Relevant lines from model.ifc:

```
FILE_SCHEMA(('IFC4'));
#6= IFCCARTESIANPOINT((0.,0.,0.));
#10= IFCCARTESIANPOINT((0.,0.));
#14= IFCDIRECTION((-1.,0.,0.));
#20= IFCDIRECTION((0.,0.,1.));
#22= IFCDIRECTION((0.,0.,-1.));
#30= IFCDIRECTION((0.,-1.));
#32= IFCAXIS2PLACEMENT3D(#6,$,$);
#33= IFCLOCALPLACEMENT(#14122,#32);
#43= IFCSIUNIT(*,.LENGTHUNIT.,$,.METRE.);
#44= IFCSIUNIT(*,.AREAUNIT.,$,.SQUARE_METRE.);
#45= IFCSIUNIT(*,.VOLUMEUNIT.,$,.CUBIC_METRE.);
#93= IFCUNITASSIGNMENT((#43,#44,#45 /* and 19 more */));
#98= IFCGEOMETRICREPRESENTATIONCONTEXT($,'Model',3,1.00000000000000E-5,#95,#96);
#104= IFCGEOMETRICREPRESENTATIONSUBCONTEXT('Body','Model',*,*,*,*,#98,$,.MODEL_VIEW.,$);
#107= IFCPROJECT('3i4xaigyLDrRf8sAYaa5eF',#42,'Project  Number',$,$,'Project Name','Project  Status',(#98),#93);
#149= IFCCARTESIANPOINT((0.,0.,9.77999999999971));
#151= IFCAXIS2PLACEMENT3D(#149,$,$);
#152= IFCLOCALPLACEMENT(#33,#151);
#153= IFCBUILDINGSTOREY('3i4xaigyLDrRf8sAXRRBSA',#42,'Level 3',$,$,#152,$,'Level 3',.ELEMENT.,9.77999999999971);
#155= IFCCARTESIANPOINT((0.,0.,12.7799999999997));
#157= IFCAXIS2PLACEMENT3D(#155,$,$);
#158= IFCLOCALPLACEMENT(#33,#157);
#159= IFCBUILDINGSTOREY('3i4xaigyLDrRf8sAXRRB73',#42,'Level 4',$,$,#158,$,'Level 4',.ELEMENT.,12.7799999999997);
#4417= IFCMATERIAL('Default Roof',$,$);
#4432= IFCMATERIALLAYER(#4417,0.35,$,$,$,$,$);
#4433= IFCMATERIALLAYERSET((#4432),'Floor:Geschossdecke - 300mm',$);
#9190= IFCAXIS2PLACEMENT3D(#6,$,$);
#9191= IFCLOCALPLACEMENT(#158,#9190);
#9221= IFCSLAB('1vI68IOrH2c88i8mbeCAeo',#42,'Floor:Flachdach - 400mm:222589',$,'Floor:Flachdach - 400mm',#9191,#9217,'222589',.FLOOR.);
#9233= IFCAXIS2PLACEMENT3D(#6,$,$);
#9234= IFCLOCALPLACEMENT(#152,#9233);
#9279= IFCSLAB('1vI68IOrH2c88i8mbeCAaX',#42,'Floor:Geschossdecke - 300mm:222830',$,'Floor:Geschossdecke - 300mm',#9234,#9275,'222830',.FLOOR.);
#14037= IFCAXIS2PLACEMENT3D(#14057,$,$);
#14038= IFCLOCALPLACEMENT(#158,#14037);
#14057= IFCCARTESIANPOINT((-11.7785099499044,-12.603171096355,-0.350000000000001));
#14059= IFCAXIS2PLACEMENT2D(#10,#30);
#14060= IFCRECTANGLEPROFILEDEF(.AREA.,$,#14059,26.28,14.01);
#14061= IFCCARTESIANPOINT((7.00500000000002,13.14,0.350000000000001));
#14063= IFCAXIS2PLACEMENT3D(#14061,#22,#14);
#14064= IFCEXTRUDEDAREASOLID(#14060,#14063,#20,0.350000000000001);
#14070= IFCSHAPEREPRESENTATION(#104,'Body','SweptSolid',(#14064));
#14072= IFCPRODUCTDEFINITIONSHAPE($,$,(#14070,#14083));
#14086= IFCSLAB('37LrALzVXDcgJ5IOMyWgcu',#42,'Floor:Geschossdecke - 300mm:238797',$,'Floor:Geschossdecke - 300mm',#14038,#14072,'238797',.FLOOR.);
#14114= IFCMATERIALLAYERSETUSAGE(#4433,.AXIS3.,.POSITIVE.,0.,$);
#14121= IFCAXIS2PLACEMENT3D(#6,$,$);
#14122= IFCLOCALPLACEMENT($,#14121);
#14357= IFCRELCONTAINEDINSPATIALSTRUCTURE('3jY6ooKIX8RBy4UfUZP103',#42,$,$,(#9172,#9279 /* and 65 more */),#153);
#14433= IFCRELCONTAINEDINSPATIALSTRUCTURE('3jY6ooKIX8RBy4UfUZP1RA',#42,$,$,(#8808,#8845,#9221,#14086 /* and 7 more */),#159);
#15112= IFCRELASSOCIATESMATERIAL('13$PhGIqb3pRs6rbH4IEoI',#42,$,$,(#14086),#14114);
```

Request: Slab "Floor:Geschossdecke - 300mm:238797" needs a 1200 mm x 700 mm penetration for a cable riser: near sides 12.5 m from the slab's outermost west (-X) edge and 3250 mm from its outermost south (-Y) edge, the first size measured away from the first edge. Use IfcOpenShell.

```python
import numpy as np
import ifcopenshell
import ifcopenshell.api.feature
import ifcopenshell.api.geometry
import ifcopenshell.api.root
import ifcopenshell.geom
import ifcopenshell.util.placement
import ifcopenshell.util.representation
import ifcopenshell.util.shape
import ifcopenshell.util.unit

model = ifcopenshell.open("model.ifc")
unit_scale = ifcopenshell.util.unit.calculate_unit_scale(model)
settings = ifcopenshell.geom.settings()


def volume(element):
    """Net volume in cubic metres, openings subtracted."""
    shape = ifcopenshell.geom.create_shape(settings, element)
    return ifcopenshell.util.shape.get_volume(shape.geometry)


slab = model.by_guid("37LrALzVXDcgJ5IOMyWgcu")
before = volume(slab)

# Extent in the slab's own axes, in metres. The edges named are its -X and -Y sides.
slab_shape = ifcopenshell.geom.create_shape(settings, slab)
vertices = ifcopenshell.util.shape.get_vertices(slab_shape.geometry)
x_min, y_min, bottom = vertices.min(axis=0)
top = vertices[:, 2].max()

opening = ifcopenshell.api.root.create_entity(model, ifc_class="IfcOpeningElement", name="Cable riser opening", predefined_type="OPENING")
context = ifcopenshell.util.representation.get_context(model, "Model", "Body", "MODEL_VIEW")
width, depth = 1.2, 0.7
outline = [(0.0, 0.0), (width, 0.0), (width, depth), (0.0, depth), (0.0, 0.0)]
# Overshoot both faces by 50 mm so the cut is clean.
shape = ifcopenshell.api.geometry.add_slab_representation(
    model, context=context, depth=top - bottom + 0.1, polyline=outline
)
ifcopenshell.api.geometry.assign_representation(model, product=opening, representation=shape)

matrix = ifcopenshell.util.placement.get_local_placement(slab.ObjectPlacement)
matrix[:, 3] = matrix @ np.append(np.array([x_min + 12.5, y_min + 3.25, bottom - 0.05]) / unit_scale, 1.0)
ifcopenshell.api.geometry.edit_object_placement(model, product=opening, matrix=matrix, is_si=False)
ifcopenshell.api.feature.add_feature(model, feature=opening, element=slab)

after = volume(slab)

print(f"slab volume {before:.3f} -> {after:.3f} m3")

model.write("model_updated.ifc")
```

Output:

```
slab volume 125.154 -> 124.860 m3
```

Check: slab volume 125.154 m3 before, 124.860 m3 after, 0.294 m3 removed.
